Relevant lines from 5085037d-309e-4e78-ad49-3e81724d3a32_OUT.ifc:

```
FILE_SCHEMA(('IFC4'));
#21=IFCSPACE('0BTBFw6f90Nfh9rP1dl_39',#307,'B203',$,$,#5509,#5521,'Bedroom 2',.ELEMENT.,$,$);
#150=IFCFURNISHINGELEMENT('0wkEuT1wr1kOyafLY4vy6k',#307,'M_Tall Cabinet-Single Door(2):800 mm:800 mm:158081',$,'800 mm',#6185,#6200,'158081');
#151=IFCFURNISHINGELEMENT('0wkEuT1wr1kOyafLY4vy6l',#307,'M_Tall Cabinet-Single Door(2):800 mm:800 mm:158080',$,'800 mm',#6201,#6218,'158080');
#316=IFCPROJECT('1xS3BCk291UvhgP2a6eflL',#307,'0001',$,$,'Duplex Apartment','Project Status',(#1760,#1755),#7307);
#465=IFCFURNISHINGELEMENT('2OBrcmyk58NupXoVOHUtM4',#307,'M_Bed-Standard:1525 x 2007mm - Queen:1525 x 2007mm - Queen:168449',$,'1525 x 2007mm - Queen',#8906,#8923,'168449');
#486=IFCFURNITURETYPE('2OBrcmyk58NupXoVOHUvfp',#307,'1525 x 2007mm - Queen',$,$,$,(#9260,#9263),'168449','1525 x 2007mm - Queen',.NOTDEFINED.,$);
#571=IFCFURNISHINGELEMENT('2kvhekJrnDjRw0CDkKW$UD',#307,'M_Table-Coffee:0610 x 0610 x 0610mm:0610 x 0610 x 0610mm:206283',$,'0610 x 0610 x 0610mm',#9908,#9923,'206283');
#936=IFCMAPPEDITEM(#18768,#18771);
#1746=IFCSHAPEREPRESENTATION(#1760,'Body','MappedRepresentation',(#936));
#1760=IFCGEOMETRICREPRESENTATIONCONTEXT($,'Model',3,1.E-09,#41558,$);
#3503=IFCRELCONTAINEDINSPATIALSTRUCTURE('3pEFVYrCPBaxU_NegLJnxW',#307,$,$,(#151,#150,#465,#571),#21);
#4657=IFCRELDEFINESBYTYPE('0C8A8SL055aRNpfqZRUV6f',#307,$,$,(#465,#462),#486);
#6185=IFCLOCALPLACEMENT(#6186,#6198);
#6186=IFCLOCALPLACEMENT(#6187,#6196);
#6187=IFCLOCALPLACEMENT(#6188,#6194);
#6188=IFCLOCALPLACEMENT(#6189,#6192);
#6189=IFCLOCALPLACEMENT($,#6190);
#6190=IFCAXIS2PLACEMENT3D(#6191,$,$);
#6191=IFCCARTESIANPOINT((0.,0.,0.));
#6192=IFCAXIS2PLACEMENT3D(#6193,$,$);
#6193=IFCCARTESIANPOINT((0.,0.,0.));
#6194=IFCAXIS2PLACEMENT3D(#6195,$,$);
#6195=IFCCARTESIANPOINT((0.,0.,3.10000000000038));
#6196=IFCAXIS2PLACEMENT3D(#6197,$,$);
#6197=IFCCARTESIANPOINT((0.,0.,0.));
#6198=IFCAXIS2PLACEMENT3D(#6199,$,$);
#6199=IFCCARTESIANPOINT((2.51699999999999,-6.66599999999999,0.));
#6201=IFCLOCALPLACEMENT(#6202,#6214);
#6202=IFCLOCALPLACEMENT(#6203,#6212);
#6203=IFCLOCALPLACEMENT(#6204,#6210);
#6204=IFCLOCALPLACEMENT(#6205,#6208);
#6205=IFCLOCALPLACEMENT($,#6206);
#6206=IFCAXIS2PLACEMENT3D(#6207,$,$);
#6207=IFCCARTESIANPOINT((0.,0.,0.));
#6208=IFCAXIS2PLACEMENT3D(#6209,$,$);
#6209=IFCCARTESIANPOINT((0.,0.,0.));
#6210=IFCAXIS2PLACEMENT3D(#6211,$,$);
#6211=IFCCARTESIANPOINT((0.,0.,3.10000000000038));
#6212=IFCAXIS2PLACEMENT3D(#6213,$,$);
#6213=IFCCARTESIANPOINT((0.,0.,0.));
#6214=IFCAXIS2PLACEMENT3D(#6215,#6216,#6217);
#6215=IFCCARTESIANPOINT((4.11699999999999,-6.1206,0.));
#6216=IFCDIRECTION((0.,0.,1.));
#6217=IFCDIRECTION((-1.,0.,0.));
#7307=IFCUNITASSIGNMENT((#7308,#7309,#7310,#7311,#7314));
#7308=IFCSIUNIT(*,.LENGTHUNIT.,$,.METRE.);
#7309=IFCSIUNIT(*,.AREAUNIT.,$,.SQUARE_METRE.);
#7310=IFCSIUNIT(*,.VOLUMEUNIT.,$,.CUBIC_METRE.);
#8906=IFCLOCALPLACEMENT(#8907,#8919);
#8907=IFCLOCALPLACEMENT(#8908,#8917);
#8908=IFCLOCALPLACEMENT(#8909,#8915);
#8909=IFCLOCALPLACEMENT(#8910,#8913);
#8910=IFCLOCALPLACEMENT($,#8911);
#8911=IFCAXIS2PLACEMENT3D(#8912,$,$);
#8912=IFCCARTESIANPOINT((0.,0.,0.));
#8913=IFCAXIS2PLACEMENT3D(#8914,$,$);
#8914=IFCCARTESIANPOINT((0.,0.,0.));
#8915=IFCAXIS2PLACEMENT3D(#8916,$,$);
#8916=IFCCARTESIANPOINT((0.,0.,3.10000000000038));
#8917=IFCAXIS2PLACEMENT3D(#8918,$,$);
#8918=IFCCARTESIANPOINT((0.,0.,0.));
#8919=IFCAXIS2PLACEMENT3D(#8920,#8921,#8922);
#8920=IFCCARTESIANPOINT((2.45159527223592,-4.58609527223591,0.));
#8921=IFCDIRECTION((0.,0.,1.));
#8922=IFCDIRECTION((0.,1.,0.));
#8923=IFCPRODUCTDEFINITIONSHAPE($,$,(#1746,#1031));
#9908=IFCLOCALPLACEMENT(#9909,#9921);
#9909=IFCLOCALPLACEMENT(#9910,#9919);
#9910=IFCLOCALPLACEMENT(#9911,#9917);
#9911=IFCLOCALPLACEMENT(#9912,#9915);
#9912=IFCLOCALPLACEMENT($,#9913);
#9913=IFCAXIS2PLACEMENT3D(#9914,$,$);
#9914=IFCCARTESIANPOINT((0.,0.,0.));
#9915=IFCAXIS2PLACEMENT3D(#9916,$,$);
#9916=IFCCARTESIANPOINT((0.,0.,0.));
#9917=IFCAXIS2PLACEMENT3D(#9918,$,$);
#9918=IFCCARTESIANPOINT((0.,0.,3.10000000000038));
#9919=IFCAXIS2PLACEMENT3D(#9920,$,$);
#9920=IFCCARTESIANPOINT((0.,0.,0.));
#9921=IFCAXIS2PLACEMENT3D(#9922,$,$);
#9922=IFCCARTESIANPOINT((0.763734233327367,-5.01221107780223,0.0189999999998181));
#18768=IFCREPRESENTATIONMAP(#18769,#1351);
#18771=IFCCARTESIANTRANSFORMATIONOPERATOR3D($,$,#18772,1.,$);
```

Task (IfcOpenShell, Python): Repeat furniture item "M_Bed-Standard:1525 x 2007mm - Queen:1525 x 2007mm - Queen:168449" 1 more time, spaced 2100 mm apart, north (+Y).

```python
import numpy as np
import ifcopenshell
import ifcopenshell.api.geometry
import ifcopenshell.api.root
import ifcopenshell.util.element
import ifcopenshell.util.placement
import ifcopenshell.util.unit

model = ifcopenshell.open("5085037d-309e-4e78-ad49-3e81724d3a32_OUT.ifc")
unit_scale = ifcopenshell.util.unit.calculate_unit_scale(model)


def reuse_history(source, copy):
    """copy_class also copies each property set's owner history, people and application; keep the originals."""
    for rel in copy.IsDefinedBy:
        if rel.is_a("IfcRelDefinesByProperties") and (history := rel.RelatingPropertyDefinition.OwnerHistory):
            rel.RelatingPropertyDefinition.OwnerHistory = source.OwnerHistory
            ifcopenshell.util.element.remove_deep2(model, history)


source = model.by_id(465)
base = ifcopenshell.util.placement.get_local_placement(source.ObjectPlacement)
step = np.array([0.0, 1.0, 0.0]) * 2.1 / unit_scale

for i in range(1, 2):
    copy = ifcopenshell.api.root.copy_class(model, product=source)
    copy.Representation = ifcopenshell.util.element.copy_deep(
        model, source.Representation, exclude=["IfcGeometricRepresentationContext", "IfcRepresentationMap"]
    )
    copy.Name = "M_Bed-Standard:1525 x 2007mm - Queen:1525 x 2007mm - Queen"
    copy.Tag = None
    reuse_history(source, copy)
    matrix = base.copy()
    matrix[:3, 3] += i * step
    print("added at", matrix[:3, 3].round(3) + 0.0)
    ifcopenshell.api.geometry.edit_object_placement(model, product=copy, matrix=matrix, is_si=False)

model.write("5085037d-309e-4e78-ad49-3e81724d3a32_OUT_edited.ifc")
```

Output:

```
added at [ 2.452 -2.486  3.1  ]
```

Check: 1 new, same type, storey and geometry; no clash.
